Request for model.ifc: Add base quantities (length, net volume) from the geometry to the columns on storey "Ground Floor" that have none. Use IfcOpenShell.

First a look at what the model holds.

```python
import ifcopenshell
import ifcopenshell.util.element
import ifcopenshell.util.unit

model = ifcopenshell.open("model.ifc")
print(model.schema)
for unit_type in ("LENGTHUNIT", "AREAUNIT", "VOLUMEUNIT"):
    print(unit_type, ifcopenshell.util.unit.calculate_unit_scale(model, unit_type))
storey = next(s for s in model.by_type("IfcBuildingStorey") if s.Name == "Ground Floor")
columns = [e for e in ifcopenshell.util.element.get_decomposition(storey) if e.is_a("IfcColumn")]
for e in sorted(columns, key=lambda e: e.id()):
    print(e.id(), e.is_a(), e.Name, list(ifcopenshell.util.element.get_psets(e, qtos_only=True)), sep=" | ")
```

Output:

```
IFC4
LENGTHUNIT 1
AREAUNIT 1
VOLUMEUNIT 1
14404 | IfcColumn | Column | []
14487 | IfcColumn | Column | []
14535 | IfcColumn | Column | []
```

```python
import ifcopenshell
import ifcopenshell.api.pset
import ifcopenshell.geom
import ifcopenshell.util.element
import ifcopenshell.util.shape
import ifcopenshell.util.unit

model = ifcopenshell.open("model.ifc")
unit_scale = ifcopenshell.util.unit.calculate_unit_scale(model)
volume_scale = ifcopenshell.util.unit.calculate_unit_scale(model, "VOLUMEUNIT")
settings = ifcopenshell.geom.settings()

storey = next(s for s in model.by_type("IfcBuildingStorey") if s.Name == "Ground Floor")
columns = [e for e in ifcopenshell.util.element.get_decomposition(storey) if e.is_a("IfcColumn")]

for e in sorted(columns, key=lambda e: e.id()):
    if ifcopenshell.util.element.get_psets(e, qtos_only=True, should_inherit=False):
        continue
    # Geometry comes back in metres, in the element's own axes.
    shape = ifcopenshell.geom.create_shape(settings, e)
    values = {
        "Length": ifcopenshell.util.shape.get_z(shape.geometry) / unit_scale,
        "NetVolume": ifcopenshell.util.shape.get_volume(shape.geometry) / volume_scale,
    }
    qto = ifcopenshell.api.pset.add_qto(model, product=e, name="Qto_ColumnBaseQuantities")
    ifcopenshell.api.pset.edit_qto(model, qto=qto, properties=values)
    print(e.id(), {k: round(v, 3) for k, v in values.items()})

model.write("model_edited.ifc")
```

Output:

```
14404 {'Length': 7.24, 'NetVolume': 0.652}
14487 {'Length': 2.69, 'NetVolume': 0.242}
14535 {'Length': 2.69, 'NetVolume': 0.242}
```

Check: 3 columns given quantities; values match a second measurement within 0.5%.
